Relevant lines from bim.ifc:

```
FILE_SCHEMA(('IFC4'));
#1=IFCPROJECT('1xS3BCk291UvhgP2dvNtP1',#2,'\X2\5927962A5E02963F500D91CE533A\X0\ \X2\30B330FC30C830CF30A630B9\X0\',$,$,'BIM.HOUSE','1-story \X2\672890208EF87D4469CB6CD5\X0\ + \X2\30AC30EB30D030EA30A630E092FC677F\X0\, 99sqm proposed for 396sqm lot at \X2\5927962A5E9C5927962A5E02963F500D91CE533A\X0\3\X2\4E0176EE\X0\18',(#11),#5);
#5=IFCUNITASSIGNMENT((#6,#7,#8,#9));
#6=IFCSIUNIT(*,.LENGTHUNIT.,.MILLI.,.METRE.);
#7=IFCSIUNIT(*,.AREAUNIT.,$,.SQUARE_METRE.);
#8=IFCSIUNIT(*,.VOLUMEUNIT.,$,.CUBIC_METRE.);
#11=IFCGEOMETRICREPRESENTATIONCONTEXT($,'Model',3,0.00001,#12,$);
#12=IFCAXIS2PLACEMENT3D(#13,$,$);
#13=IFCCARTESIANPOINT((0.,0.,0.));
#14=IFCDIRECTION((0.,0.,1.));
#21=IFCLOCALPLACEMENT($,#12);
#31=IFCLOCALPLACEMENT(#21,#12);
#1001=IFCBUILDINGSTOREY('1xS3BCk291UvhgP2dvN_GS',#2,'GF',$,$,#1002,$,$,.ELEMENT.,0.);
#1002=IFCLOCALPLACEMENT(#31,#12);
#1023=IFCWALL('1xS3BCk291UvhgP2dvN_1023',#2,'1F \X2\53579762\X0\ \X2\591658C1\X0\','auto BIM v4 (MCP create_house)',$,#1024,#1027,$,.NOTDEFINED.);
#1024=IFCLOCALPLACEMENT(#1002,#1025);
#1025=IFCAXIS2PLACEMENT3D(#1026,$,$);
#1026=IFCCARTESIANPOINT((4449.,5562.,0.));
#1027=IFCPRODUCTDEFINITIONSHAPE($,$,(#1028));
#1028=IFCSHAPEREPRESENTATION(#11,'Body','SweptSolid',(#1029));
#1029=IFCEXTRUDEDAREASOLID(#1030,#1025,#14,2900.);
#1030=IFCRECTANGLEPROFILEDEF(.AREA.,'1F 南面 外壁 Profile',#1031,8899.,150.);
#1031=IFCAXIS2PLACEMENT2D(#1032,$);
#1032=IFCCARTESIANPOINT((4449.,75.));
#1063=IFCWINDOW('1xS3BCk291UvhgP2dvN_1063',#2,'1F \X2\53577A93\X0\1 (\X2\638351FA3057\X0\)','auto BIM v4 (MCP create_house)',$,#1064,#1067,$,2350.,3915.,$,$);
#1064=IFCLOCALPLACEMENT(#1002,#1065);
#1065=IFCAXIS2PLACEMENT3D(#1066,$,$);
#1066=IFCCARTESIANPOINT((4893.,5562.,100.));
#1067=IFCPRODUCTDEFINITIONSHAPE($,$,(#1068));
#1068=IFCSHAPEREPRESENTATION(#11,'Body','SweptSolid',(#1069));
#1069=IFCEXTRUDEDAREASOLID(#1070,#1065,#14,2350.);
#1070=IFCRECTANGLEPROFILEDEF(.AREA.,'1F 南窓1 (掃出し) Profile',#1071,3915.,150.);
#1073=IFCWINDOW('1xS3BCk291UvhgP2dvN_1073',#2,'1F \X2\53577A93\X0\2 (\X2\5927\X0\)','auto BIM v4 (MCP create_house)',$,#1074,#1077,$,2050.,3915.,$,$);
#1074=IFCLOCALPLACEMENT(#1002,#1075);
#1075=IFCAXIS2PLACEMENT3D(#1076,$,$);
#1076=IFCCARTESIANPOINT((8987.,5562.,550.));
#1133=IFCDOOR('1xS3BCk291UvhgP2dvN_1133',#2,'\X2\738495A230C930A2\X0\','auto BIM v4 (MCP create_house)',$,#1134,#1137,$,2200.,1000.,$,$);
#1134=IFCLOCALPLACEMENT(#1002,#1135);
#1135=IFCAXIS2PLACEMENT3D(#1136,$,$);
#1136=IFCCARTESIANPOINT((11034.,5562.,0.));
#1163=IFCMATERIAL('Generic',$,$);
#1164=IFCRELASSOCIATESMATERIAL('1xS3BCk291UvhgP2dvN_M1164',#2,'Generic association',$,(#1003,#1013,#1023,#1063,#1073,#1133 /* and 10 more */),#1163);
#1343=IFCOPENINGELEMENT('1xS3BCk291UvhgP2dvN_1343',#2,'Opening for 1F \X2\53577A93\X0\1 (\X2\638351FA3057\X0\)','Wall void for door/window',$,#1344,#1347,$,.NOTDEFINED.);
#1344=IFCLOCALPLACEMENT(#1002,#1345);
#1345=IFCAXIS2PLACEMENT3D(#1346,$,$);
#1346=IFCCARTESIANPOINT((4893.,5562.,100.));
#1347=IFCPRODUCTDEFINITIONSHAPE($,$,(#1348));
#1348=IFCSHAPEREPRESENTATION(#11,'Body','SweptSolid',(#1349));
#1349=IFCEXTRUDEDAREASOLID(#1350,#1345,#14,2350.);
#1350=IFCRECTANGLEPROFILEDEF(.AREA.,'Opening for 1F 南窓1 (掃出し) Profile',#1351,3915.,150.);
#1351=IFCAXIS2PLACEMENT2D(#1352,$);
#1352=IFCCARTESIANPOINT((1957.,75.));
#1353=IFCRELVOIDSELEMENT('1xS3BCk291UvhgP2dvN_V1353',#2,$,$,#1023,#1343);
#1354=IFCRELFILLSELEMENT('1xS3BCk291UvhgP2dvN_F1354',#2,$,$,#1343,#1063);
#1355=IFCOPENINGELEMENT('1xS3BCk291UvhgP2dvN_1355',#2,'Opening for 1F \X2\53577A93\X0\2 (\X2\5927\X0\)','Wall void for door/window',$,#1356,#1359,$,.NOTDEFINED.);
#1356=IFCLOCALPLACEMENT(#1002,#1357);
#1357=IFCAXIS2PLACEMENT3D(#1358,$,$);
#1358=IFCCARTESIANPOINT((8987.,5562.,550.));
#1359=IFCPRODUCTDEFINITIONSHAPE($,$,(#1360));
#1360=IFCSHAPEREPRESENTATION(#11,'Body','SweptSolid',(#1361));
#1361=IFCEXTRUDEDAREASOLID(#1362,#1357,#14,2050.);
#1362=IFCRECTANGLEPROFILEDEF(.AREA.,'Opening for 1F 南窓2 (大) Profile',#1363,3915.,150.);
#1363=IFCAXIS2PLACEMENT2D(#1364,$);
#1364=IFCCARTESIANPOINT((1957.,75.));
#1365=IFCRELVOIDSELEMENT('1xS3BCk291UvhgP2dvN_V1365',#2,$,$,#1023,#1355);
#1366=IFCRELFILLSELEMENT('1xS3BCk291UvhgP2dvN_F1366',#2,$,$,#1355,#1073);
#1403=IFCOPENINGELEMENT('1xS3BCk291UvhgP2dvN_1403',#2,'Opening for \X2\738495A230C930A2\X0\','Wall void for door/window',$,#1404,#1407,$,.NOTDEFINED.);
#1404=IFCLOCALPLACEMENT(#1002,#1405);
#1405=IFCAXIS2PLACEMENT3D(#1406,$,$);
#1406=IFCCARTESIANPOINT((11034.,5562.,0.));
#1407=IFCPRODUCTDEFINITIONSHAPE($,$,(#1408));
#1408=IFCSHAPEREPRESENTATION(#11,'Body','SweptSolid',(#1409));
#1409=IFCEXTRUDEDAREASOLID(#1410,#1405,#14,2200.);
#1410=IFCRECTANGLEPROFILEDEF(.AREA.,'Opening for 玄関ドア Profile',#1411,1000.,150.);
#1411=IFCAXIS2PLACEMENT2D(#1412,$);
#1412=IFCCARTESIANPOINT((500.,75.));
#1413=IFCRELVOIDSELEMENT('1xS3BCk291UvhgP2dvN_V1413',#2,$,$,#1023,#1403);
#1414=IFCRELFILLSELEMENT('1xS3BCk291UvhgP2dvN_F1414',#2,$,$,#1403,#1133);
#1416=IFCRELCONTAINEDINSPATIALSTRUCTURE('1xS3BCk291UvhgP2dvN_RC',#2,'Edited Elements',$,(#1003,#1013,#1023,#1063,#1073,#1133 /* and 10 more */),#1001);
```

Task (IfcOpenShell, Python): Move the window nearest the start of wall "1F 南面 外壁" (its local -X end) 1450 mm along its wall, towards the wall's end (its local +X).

```python
import ifcopenshell
import ifcopenshell.api.geometry
import ifcopenshell.util.placement
import ifcopenshell.util.unit

model = ifcopenshell.open("bim.ifc")
unit_scale = ifcopenshell.util.unit.calculate_unit_scale(model)

window = model.by_guid("1xS3BCk291UvhgP2dvN_1063")
opening = window.FillsVoids[0].RelatingOpeningElement
wall = opening.VoidsElements[0].RelatingBuildingElement

wall_matrix = ifcopenshell.util.placement.get_local_placement(wall.ObjectPlacement)
shift = wall_matrix[:3, 0] * 1.45 / unit_scale
before = ifcopenshell.util.placement.get_local_placement(window.ObjectPlacement)[:3, 3].copy()

# The window is not placed relative to its opening, so move both.
for product in (opening, window):
    matrix = ifcopenshell.util.placement.get_local_placement(product.ObjectPlacement)
    matrix[:3, 3] += shift
    ifcopenshell.api.geometry.edit_object_placement(model, product=product, matrix=matrix, is_si=False)

after = ifcopenshell.util.placement.get_local_placement(window.ObjectPlacement)[:3, 3]
print("window moved by", (after - before).round(3) + 0.0)

model.write("bim_edited.ifc")
```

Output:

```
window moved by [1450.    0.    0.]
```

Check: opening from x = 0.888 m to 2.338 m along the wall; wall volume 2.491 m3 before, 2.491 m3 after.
